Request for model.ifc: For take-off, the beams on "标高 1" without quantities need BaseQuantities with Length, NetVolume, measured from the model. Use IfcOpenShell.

First a look at what the model holds.

```python
import ifcopenshell
import ifcopenshell.util.element
import ifcopenshell.util.unit

model = ifcopenshell.open("model.ifc")
print(model.schema)
for unit_type in ("LENGTHUNIT", "AREAUNIT", "VOLUMEUNIT"):
    print(unit_type, ifcopenshell.util.unit.calculate_unit_scale(model, unit_type))
storey = next(s for s in model.by_type("IfcBuildingStorey") if s.Name == "标高 1")
beams = [e for e in ifcopenshell.util.element.get_decomposition(storey) if e.is_a("IfcBeam")]
for e in sorted(beams, key=lambda e: e.id()):
    print(e.id(), e.is_a(), e.Name, list(ifcopenshell.util.element.get_psets(e, qtos_only=True)), sep=" | ")
```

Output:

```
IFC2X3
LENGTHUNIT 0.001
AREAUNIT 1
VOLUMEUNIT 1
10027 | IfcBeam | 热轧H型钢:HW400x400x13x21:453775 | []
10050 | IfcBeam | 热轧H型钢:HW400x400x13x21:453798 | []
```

```python
import ifcopenshell
import ifcopenshell.api.pset
import ifcopenshell.geom
import ifcopenshell.util.element
import ifcopenshell.util.shape
import ifcopenshell.util.unit

model = ifcopenshell.open("model.ifc")
unit_scale = ifcopenshell.util.unit.calculate_unit_scale(model)
volume_scale = ifcopenshell.util.unit.calculate_unit_scale(model, "VOLUMEUNIT")
settings = ifcopenshell.geom.settings()

storey = next(s for s in model.by_type("IfcBuildingStorey") if s.Name == "标高 1")
beams = [e for e in ifcopenshell.util.element.get_decomposition(storey) if e.is_a("IfcBeam")]

for e in sorted(beams, key=lambda e: e.id()):
    if ifcopenshell.util.element.get_psets(e, qtos_only=True, should_inherit=False):
        continue
    # Geometry comes back in metres, in the element's own axes.
    shape = ifcopenshell.geom.create_shape(settings, e)
    values = {
        "Length": ifcopenshell.util.shape.get_max_xyz(shape.geometry) / unit_scale,
        "NetVolume": ifcopenshell.util.shape.get_volume(shape.geometry) / volume_scale,
    }
    qto = ifcopenshell.api.pset.add_qto(model, product=e, name="BaseQuantities")
    ifcopenshell.api.pset.edit_qto(model, qto=qto, properties=values)
    print(e.id(), {k: round(v, 3) for k, v in values.items()})

model.write("model_v2.ifc")
```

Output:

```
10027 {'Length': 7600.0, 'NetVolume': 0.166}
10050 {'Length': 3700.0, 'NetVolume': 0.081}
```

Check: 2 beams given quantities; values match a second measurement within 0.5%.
